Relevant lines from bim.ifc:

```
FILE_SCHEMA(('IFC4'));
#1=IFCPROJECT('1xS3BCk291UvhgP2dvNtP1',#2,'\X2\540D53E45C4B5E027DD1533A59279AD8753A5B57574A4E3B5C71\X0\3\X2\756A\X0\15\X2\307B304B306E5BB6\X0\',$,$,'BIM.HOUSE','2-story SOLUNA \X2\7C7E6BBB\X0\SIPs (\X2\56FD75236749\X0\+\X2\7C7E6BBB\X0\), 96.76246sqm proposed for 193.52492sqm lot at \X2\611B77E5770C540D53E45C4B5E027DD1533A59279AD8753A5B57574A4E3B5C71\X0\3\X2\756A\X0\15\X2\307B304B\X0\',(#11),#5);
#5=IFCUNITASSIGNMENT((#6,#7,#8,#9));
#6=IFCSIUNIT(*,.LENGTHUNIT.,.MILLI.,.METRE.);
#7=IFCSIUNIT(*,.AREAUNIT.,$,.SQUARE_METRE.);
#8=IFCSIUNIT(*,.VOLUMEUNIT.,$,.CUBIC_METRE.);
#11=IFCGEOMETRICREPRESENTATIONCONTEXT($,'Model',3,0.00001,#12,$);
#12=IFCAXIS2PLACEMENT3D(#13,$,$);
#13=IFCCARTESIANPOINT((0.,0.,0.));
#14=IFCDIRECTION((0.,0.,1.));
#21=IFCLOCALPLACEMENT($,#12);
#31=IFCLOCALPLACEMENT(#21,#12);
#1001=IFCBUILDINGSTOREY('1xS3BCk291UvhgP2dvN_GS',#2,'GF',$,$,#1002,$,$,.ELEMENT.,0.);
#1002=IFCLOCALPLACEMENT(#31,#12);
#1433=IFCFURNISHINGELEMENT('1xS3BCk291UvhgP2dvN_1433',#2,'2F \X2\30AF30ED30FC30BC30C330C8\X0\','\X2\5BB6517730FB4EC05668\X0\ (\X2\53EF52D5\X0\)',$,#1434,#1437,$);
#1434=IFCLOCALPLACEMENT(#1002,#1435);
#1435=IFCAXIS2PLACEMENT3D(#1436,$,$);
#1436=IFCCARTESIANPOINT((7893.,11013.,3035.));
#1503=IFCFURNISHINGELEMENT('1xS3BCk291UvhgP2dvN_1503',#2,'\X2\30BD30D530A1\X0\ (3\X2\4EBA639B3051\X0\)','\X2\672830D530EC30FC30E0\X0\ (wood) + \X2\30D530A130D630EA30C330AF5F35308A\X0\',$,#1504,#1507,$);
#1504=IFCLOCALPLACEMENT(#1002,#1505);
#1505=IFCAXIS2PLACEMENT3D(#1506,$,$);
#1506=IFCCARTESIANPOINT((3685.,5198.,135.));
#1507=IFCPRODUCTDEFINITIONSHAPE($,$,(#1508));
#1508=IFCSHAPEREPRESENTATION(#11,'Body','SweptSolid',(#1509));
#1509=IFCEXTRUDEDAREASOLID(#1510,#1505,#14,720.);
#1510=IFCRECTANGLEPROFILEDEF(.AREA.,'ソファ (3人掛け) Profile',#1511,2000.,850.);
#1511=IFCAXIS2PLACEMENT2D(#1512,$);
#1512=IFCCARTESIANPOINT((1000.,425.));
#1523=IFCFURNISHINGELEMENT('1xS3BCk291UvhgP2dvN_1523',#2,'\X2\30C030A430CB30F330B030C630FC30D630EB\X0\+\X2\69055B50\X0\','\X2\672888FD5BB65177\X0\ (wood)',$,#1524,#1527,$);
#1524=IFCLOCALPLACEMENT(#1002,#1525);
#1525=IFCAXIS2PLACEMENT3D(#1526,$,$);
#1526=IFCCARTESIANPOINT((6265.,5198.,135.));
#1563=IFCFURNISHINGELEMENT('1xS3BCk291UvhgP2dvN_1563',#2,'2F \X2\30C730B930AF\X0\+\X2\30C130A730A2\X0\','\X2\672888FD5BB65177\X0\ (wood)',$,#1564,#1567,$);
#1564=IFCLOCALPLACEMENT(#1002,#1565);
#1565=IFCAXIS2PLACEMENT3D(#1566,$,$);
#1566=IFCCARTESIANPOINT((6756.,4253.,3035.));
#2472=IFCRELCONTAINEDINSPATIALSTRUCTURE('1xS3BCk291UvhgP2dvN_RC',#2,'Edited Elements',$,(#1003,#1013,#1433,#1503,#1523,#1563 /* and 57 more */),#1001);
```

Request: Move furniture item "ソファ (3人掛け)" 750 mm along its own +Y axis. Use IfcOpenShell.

```python
import ifcopenshell
import ifcopenshell.api.geometry
import ifcopenshell.util.placement
import ifcopenshell.util.unit

model = ifcopenshell.open("bim.ifc")
unit_scale = ifcopenshell.util.unit.calculate_unit_scale(model)

item = model.by_guid("1xS3BCk291UvhgP2dvN_1503")
matrix = ifcopenshell.util.placement.get_local_placement(item.ObjectPlacement)
matrix[:3, 3] += matrix[:3, 1] * 0.75 / unit_scale
ifcopenshell.api.geometry.edit_object_placement(model, product=item, matrix=matrix, is_si=False)

print(ifcopenshell.util.placement.get_local_placement(item.ObjectPlacement).round(3) + 0.0)

model.write("bim_edited.ifc")
```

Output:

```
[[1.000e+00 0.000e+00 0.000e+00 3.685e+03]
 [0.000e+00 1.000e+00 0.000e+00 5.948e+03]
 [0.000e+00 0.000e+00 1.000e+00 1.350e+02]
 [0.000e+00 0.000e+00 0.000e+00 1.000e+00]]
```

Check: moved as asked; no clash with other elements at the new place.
